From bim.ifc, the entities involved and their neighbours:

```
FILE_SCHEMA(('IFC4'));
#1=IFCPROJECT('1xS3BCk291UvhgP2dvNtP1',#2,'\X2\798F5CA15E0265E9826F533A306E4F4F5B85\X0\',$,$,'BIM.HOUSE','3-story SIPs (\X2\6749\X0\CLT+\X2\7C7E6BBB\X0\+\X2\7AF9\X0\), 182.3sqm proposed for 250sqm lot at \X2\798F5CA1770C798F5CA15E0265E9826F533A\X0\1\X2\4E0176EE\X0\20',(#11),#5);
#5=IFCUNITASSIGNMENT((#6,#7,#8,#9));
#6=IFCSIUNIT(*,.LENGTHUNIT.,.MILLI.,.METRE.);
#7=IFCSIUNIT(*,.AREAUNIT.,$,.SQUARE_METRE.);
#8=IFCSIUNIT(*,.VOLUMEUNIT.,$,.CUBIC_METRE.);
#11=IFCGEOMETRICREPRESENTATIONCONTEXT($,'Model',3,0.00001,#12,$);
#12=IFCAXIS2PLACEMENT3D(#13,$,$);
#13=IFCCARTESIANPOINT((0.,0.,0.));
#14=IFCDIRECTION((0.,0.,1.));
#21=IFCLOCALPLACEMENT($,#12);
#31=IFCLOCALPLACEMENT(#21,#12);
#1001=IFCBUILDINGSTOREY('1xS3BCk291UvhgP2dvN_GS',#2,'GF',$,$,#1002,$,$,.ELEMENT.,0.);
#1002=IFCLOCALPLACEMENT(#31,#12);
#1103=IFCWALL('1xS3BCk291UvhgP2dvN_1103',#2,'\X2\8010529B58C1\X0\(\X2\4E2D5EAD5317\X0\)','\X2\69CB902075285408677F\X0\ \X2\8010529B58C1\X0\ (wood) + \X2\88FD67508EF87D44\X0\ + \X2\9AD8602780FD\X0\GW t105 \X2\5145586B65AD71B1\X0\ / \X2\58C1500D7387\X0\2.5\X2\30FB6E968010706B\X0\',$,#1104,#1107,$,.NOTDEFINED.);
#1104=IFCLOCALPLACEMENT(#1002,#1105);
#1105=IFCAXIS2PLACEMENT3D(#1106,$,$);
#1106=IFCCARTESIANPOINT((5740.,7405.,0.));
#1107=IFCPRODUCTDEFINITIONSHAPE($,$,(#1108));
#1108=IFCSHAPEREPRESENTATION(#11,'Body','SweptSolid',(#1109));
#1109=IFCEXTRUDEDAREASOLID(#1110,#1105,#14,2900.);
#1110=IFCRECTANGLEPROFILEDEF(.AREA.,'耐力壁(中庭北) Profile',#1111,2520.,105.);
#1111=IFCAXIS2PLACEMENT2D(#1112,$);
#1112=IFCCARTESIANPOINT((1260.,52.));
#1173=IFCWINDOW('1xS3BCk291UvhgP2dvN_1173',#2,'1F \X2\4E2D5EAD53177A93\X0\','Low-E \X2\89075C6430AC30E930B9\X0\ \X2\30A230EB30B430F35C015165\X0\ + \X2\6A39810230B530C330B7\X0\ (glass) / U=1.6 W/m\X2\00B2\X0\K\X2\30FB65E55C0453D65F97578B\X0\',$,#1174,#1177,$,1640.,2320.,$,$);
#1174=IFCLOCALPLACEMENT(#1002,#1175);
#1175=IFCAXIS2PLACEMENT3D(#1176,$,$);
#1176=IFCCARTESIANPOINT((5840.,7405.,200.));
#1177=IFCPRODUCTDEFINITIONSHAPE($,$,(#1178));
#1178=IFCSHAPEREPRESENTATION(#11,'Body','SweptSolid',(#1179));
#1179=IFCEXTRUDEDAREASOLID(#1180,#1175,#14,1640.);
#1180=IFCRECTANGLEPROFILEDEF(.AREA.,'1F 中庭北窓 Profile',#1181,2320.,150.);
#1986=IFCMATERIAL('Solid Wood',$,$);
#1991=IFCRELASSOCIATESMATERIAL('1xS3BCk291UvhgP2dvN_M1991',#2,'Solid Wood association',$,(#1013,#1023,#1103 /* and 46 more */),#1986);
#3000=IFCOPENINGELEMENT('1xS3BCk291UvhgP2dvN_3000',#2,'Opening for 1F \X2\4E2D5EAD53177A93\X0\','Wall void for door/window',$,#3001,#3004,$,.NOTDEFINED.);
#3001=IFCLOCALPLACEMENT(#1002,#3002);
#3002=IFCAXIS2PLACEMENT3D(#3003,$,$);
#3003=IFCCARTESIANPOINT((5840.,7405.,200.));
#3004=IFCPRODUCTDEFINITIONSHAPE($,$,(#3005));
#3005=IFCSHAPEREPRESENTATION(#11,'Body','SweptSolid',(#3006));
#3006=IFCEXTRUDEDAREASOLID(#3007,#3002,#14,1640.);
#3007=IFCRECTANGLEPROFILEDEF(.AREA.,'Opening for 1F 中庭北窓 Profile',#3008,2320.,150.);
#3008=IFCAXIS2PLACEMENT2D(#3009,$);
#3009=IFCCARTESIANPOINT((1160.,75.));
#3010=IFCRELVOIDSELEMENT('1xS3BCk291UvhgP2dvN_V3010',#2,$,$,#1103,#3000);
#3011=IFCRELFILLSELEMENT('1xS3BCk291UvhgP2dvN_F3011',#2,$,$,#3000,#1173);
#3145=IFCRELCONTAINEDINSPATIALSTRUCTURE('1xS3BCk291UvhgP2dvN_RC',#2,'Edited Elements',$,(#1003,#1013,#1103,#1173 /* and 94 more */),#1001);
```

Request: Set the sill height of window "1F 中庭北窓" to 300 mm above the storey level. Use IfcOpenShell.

```python
import numpy as np
import ifcopenshell
import ifcopenshell.api.geometry
import ifcopenshell.geom
import ifcopenshell.util.element
import ifcopenshell.util.placement
import ifcopenshell.util.shape
import ifcopenshell.util.unit

model = ifcopenshell.open("bim.ifc")
unit_scale = ifcopenshell.util.unit.calculate_unit_scale(model)

window = model.by_guid("1xS3BCk291UvhgP2dvN_1173")
opening = window.FillsVoids[0].RelatingOpeningElement
storey = ifcopenshell.util.element.get_container(window, ifc_class="IfcBuildingStorey")
level = ifcopenshell.util.placement.get_local_placement(storey.ObjectPlacement)[2, 3]

# The opening's origin need not be at the sill, so measure its lowest point.
shape = ifcopenshell.geom.create_shape(ifcopenshell.geom.settings(), opening)
bottom = ifcopenshell.util.shape.get_shape_bottom_elevation(shape, shape.geometry) / unit_scale
dz = level + 0.3 / unit_scale - bottom

shift = np.array([0.0, 0.0, dz])
# The window is not placed relative to its opening, so move both.
for product in (opening, window):
    matrix = ifcopenshell.util.placement.get_local_placement(product.ObjectPlacement)
    matrix[:3, 3] += shift
    ifcopenshell.api.geometry.edit_object_placement(model, product=product, matrix=matrix, is_si=False)

print(f"moved by {dz * unit_scale:+.3f} m")

model.write("bim_v2.ifc")
```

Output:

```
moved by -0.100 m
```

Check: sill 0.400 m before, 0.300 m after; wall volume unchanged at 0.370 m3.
